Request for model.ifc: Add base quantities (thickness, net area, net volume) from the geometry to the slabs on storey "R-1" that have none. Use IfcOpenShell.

First a look at what the model holds.

```python
import ifcopenshell
import ifcopenshell.util.element
import ifcopenshell.util.unit

model = ifcopenshell.open("model.ifc")
print(model.schema)
for unit_type in ("LENGTHUNIT", "AREAUNIT", "VOLUMEUNIT"):
    print(unit_type, ifcopenshell.util.unit.calculate_unit_scale(model, unit_type))
storey = next(s for s in model.by_type("IfcBuildingStorey") if s.Name == "R-1")
slabs = [e for e in ifcopenshell.util.element.get_decomposition(storey) if e.is_a("IfcSlab")]
for e in sorted(slabs, key=lambda e: e.id()):
    print(e.id(), e.is_a(), e.Name, list(ifcopenshell.util.element.get_psets(e, qtos_only=True)), sep=" | ")
```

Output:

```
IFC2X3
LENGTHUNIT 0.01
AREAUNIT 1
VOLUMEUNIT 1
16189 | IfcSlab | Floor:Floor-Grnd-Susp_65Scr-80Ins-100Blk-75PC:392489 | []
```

```python
import ifcopenshell
import ifcopenshell.api.pset
import ifcopenshell.geom
import ifcopenshell.util.element
import ifcopenshell.util.shape
import ifcopenshell.util.unit

model = ifcopenshell.open("model.ifc")
unit_scale = ifcopenshell.util.unit.calculate_unit_scale(model)
area_scale = ifcopenshell.util.unit.calculate_unit_scale(model, "AREAUNIT")
volume_scale = ifcopenshell.util.unit.calculate_unit_scale(model, "VOLUMEUNIT")
settings = ifcopenshell.geom.settings()

storey = next(s for s in model.by_type("IfcBuildingStorey") if s.Name == "R-1")
slabs = [e for e in ifcopenshell.util.element.get_decomposition(storey) if e.is_a("IfcSlab")]

for e in sorted(slabs, key=lambda e: e.id()):
    if ifcopenshell.util.element.get_psets(e, qtos_only=True, should_inherit=False):
        continue
    # Geometry comes back in metres, in the element's own axes.
    shape = ifcopenshell.geom.create_shape(settings, e)
    values = {
        "Width": ifcopenshell.util.shape.get_z(shape.geometry) / unit_scale,
        "NetArea": ifcopenshell.util.shape.get_footprint_area(shape.geometry) / area_scale,
        "NetVolume": ifcopenshell.util.shape.get_volume(shape.geometry) / volume_scale,
    }
    qto = ifcopenshell.api.pset.add_qto(model, product=e, name="BaseQuantities")
    ifcopenshell.api.pset.edit_qto(model, qto=qto, properties=values)
    print(e.id(), {k: round(v, 3) for k, v in values.items()})

model.write("model_updated.ifc")
```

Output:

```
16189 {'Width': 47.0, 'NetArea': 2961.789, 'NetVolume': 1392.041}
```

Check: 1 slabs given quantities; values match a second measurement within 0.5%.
